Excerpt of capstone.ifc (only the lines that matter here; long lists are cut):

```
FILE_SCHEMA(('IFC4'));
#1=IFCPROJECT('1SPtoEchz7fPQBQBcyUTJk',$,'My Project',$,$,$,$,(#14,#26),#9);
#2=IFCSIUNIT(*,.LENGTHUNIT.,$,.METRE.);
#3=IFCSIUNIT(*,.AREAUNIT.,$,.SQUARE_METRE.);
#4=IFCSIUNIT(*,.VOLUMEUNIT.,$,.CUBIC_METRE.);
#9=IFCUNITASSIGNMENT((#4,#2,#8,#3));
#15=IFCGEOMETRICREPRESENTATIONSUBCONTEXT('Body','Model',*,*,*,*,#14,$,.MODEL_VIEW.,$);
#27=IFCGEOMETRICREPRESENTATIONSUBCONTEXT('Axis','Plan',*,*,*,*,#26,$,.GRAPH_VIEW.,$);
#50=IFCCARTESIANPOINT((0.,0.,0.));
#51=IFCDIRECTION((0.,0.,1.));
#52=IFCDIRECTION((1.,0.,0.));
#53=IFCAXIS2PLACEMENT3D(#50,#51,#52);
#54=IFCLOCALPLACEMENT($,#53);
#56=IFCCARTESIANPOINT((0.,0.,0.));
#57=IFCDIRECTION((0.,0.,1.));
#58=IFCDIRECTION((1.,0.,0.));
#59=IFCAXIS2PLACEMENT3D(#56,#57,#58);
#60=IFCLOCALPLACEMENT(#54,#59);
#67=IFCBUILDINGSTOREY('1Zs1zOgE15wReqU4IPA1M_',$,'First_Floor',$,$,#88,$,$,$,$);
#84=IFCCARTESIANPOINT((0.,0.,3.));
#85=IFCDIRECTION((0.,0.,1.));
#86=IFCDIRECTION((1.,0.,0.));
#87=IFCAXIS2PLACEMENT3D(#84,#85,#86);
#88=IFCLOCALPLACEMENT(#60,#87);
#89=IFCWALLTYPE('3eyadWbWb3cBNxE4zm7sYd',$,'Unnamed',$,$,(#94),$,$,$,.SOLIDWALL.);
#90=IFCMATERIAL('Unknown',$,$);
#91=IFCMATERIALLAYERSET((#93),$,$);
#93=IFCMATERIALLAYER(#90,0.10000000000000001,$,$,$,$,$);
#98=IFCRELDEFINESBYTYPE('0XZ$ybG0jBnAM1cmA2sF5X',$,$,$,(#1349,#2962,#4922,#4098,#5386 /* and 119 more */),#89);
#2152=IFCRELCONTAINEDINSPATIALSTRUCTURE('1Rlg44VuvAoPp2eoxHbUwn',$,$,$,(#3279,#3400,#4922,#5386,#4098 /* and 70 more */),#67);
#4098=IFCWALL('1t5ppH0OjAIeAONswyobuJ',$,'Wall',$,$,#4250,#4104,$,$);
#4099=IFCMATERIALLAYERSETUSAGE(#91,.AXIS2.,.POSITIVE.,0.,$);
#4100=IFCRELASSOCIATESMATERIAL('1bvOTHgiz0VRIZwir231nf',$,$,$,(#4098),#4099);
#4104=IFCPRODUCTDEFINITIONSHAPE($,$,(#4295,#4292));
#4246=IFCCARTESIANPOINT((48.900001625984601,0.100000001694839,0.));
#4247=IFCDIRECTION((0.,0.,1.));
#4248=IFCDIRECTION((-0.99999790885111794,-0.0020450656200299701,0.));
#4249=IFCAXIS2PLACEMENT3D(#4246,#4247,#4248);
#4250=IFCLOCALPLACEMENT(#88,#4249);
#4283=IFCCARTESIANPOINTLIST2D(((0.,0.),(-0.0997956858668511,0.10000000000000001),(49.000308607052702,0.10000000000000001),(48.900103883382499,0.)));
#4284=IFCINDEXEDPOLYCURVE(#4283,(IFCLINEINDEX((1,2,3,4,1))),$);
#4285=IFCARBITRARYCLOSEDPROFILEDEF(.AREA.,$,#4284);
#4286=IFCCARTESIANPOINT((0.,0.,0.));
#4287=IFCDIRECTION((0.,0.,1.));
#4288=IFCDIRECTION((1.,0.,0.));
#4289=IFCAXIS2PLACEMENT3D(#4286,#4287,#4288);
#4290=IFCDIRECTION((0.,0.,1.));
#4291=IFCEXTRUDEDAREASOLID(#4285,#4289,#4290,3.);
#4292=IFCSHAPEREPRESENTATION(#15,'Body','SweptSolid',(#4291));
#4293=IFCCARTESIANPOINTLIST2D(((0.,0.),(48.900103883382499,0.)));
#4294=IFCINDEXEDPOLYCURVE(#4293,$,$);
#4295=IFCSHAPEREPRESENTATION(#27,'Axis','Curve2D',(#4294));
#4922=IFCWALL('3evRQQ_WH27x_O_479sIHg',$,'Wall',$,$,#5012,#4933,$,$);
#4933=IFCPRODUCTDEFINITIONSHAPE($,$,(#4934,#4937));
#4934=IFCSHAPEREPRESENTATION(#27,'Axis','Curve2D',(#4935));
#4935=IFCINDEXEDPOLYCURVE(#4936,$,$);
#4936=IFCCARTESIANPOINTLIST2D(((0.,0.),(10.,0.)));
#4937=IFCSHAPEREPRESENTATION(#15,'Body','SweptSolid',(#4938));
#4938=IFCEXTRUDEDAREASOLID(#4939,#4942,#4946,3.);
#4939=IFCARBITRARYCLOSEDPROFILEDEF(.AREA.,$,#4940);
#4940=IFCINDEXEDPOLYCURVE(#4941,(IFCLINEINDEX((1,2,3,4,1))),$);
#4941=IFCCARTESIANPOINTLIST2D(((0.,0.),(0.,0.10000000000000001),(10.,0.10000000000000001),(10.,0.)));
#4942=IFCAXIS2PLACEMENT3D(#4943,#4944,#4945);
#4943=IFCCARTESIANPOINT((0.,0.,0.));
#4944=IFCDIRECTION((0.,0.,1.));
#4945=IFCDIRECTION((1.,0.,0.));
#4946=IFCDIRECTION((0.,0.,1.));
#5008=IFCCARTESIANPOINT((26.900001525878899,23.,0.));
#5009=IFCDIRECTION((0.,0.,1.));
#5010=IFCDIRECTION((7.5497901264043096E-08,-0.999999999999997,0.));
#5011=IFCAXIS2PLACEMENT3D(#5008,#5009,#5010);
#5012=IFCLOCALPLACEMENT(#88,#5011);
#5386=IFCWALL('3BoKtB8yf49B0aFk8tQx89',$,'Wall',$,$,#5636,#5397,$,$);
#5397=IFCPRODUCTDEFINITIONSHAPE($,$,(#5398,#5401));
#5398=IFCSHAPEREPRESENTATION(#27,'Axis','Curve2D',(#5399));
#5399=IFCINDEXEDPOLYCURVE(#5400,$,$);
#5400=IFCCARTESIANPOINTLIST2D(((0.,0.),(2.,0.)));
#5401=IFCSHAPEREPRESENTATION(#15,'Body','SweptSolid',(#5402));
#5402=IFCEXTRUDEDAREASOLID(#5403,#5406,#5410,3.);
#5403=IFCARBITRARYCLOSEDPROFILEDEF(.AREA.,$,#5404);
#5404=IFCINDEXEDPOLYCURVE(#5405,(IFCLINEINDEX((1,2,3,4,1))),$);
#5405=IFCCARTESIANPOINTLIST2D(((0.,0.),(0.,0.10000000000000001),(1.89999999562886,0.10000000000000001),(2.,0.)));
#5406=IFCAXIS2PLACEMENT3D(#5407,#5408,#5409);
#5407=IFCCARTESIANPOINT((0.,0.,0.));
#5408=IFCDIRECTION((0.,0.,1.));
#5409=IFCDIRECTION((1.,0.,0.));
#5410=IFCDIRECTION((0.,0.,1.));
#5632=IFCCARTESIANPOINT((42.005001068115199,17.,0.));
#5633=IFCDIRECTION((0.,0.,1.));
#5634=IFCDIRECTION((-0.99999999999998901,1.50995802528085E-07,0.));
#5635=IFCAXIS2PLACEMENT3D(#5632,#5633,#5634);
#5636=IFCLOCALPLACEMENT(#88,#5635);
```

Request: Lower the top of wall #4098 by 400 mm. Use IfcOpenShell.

```python
import ifcopenshell
import ifcopenshell.geom
import ifcopenshell.util.representation
import ifcopenshell.util.shape
import ifcopenshell.util.unit

model = ifcopenshell.open("capstone.ifc")
unit_scale = ifcopenshell.util.unit.calculate_unit_scale(model)
settings = ifcopenshell.geom.settings()


def volume(element):
    """Net volume in cubic metres, openings subtracted."""
    shape = ifcopenshell.geom.create_shape(settings, element)
    return ifcopenshell.util.shape.get_volume(shape.geometry)


wall = model.by_guid("1t5ppH0OjAIeAONswyobuJ")
before = volume(wall)

body = ifcopenshell.util.representation.get_representation(wall, "Model", "Body")
solid = body.Items[0]
old_height = solid.Depth
solid.Depth -= 0.4 / unit_scale
after = volume(wall)

print(f"height {old_height:g} -> {solid.Depth:g}, volume {before:.3f} -> {after:.3f} m3")

model.write("capstone_edited.ifc")
```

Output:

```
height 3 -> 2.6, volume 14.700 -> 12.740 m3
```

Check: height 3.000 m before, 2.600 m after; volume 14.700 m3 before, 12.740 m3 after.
